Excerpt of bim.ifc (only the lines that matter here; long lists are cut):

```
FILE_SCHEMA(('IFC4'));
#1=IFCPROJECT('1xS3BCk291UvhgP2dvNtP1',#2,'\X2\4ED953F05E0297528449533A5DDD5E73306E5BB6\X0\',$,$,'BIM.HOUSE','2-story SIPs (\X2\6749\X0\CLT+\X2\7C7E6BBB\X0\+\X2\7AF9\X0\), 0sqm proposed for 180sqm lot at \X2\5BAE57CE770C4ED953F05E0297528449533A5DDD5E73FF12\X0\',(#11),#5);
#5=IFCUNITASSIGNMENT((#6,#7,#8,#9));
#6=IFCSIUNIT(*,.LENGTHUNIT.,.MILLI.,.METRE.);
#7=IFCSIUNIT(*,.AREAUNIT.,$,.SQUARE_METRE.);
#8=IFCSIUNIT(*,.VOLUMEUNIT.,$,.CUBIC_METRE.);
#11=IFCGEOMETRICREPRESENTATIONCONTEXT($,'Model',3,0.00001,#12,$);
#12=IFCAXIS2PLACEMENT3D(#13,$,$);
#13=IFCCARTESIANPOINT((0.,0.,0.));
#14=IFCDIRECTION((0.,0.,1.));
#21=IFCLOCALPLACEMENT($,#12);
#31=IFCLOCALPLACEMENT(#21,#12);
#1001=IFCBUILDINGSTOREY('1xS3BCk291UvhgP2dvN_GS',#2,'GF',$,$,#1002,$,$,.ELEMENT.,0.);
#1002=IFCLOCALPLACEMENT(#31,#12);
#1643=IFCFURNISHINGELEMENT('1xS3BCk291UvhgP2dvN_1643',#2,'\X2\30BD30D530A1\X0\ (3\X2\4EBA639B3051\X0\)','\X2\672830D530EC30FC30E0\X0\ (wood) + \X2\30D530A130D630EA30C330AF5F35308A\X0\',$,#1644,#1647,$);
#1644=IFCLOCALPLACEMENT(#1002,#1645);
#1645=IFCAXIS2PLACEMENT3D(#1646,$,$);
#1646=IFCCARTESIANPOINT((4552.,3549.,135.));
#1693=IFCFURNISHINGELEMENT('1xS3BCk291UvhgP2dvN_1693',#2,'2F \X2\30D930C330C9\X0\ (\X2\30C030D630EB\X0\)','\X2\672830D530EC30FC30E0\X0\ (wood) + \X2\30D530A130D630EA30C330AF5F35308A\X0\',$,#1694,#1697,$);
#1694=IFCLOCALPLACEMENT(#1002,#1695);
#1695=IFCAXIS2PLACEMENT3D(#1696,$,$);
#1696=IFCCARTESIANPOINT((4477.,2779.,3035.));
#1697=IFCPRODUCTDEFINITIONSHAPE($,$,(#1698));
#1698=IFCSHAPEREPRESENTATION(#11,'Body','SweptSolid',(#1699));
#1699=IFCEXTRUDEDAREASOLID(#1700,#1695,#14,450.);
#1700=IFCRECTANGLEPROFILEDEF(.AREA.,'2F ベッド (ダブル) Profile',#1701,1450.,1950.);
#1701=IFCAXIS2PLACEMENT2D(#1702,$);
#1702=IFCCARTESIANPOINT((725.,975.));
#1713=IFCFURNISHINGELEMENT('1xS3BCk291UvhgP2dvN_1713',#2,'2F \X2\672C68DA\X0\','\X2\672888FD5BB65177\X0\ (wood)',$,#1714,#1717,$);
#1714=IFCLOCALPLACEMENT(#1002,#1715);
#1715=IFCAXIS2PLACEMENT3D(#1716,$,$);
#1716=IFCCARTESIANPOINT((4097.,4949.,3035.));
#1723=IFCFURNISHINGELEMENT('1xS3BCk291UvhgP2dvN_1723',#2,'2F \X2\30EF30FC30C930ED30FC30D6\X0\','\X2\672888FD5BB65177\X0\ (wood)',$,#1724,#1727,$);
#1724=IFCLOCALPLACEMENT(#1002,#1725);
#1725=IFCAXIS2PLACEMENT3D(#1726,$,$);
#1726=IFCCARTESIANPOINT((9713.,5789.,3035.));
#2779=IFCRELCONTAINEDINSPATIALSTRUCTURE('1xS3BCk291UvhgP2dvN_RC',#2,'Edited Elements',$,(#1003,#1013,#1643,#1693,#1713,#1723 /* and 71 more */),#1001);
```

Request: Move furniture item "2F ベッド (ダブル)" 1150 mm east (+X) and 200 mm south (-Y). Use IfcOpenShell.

```python
import ifcopenshell
import ifcopenshell.api.geometry
import ifcopenshell.util.placement
import ifcopenshell.util.unit

model = ifcopenshell.open("bim.ifc")
unit_scale = ifcopenshell.util.unit.calculate_unit_scale(model)

item = model.by_guid("1xS3BCk291UvhgP2dvN_1693")
matrix = ifcopenshell.util.placement.get_local_placement(item.ObjectPlacement)
matrix[0, 3] += 1.15 / unit_scale
matrix[1, 3] -= 0.2 / unit_scale
ifcopenshell.api.geometry.edit_object_placement(model, product=item, matrix=matrix, is_si=False)

print(ifcopenshell.util.placement.get_local_placement(item.ObjectPlacement).round(3) + 0.0)

model.write("bim_edited.ifc")
```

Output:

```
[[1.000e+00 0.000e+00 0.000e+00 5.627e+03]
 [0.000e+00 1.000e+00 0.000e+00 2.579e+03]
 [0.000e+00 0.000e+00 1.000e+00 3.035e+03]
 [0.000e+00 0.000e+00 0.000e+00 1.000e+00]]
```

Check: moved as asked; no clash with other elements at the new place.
